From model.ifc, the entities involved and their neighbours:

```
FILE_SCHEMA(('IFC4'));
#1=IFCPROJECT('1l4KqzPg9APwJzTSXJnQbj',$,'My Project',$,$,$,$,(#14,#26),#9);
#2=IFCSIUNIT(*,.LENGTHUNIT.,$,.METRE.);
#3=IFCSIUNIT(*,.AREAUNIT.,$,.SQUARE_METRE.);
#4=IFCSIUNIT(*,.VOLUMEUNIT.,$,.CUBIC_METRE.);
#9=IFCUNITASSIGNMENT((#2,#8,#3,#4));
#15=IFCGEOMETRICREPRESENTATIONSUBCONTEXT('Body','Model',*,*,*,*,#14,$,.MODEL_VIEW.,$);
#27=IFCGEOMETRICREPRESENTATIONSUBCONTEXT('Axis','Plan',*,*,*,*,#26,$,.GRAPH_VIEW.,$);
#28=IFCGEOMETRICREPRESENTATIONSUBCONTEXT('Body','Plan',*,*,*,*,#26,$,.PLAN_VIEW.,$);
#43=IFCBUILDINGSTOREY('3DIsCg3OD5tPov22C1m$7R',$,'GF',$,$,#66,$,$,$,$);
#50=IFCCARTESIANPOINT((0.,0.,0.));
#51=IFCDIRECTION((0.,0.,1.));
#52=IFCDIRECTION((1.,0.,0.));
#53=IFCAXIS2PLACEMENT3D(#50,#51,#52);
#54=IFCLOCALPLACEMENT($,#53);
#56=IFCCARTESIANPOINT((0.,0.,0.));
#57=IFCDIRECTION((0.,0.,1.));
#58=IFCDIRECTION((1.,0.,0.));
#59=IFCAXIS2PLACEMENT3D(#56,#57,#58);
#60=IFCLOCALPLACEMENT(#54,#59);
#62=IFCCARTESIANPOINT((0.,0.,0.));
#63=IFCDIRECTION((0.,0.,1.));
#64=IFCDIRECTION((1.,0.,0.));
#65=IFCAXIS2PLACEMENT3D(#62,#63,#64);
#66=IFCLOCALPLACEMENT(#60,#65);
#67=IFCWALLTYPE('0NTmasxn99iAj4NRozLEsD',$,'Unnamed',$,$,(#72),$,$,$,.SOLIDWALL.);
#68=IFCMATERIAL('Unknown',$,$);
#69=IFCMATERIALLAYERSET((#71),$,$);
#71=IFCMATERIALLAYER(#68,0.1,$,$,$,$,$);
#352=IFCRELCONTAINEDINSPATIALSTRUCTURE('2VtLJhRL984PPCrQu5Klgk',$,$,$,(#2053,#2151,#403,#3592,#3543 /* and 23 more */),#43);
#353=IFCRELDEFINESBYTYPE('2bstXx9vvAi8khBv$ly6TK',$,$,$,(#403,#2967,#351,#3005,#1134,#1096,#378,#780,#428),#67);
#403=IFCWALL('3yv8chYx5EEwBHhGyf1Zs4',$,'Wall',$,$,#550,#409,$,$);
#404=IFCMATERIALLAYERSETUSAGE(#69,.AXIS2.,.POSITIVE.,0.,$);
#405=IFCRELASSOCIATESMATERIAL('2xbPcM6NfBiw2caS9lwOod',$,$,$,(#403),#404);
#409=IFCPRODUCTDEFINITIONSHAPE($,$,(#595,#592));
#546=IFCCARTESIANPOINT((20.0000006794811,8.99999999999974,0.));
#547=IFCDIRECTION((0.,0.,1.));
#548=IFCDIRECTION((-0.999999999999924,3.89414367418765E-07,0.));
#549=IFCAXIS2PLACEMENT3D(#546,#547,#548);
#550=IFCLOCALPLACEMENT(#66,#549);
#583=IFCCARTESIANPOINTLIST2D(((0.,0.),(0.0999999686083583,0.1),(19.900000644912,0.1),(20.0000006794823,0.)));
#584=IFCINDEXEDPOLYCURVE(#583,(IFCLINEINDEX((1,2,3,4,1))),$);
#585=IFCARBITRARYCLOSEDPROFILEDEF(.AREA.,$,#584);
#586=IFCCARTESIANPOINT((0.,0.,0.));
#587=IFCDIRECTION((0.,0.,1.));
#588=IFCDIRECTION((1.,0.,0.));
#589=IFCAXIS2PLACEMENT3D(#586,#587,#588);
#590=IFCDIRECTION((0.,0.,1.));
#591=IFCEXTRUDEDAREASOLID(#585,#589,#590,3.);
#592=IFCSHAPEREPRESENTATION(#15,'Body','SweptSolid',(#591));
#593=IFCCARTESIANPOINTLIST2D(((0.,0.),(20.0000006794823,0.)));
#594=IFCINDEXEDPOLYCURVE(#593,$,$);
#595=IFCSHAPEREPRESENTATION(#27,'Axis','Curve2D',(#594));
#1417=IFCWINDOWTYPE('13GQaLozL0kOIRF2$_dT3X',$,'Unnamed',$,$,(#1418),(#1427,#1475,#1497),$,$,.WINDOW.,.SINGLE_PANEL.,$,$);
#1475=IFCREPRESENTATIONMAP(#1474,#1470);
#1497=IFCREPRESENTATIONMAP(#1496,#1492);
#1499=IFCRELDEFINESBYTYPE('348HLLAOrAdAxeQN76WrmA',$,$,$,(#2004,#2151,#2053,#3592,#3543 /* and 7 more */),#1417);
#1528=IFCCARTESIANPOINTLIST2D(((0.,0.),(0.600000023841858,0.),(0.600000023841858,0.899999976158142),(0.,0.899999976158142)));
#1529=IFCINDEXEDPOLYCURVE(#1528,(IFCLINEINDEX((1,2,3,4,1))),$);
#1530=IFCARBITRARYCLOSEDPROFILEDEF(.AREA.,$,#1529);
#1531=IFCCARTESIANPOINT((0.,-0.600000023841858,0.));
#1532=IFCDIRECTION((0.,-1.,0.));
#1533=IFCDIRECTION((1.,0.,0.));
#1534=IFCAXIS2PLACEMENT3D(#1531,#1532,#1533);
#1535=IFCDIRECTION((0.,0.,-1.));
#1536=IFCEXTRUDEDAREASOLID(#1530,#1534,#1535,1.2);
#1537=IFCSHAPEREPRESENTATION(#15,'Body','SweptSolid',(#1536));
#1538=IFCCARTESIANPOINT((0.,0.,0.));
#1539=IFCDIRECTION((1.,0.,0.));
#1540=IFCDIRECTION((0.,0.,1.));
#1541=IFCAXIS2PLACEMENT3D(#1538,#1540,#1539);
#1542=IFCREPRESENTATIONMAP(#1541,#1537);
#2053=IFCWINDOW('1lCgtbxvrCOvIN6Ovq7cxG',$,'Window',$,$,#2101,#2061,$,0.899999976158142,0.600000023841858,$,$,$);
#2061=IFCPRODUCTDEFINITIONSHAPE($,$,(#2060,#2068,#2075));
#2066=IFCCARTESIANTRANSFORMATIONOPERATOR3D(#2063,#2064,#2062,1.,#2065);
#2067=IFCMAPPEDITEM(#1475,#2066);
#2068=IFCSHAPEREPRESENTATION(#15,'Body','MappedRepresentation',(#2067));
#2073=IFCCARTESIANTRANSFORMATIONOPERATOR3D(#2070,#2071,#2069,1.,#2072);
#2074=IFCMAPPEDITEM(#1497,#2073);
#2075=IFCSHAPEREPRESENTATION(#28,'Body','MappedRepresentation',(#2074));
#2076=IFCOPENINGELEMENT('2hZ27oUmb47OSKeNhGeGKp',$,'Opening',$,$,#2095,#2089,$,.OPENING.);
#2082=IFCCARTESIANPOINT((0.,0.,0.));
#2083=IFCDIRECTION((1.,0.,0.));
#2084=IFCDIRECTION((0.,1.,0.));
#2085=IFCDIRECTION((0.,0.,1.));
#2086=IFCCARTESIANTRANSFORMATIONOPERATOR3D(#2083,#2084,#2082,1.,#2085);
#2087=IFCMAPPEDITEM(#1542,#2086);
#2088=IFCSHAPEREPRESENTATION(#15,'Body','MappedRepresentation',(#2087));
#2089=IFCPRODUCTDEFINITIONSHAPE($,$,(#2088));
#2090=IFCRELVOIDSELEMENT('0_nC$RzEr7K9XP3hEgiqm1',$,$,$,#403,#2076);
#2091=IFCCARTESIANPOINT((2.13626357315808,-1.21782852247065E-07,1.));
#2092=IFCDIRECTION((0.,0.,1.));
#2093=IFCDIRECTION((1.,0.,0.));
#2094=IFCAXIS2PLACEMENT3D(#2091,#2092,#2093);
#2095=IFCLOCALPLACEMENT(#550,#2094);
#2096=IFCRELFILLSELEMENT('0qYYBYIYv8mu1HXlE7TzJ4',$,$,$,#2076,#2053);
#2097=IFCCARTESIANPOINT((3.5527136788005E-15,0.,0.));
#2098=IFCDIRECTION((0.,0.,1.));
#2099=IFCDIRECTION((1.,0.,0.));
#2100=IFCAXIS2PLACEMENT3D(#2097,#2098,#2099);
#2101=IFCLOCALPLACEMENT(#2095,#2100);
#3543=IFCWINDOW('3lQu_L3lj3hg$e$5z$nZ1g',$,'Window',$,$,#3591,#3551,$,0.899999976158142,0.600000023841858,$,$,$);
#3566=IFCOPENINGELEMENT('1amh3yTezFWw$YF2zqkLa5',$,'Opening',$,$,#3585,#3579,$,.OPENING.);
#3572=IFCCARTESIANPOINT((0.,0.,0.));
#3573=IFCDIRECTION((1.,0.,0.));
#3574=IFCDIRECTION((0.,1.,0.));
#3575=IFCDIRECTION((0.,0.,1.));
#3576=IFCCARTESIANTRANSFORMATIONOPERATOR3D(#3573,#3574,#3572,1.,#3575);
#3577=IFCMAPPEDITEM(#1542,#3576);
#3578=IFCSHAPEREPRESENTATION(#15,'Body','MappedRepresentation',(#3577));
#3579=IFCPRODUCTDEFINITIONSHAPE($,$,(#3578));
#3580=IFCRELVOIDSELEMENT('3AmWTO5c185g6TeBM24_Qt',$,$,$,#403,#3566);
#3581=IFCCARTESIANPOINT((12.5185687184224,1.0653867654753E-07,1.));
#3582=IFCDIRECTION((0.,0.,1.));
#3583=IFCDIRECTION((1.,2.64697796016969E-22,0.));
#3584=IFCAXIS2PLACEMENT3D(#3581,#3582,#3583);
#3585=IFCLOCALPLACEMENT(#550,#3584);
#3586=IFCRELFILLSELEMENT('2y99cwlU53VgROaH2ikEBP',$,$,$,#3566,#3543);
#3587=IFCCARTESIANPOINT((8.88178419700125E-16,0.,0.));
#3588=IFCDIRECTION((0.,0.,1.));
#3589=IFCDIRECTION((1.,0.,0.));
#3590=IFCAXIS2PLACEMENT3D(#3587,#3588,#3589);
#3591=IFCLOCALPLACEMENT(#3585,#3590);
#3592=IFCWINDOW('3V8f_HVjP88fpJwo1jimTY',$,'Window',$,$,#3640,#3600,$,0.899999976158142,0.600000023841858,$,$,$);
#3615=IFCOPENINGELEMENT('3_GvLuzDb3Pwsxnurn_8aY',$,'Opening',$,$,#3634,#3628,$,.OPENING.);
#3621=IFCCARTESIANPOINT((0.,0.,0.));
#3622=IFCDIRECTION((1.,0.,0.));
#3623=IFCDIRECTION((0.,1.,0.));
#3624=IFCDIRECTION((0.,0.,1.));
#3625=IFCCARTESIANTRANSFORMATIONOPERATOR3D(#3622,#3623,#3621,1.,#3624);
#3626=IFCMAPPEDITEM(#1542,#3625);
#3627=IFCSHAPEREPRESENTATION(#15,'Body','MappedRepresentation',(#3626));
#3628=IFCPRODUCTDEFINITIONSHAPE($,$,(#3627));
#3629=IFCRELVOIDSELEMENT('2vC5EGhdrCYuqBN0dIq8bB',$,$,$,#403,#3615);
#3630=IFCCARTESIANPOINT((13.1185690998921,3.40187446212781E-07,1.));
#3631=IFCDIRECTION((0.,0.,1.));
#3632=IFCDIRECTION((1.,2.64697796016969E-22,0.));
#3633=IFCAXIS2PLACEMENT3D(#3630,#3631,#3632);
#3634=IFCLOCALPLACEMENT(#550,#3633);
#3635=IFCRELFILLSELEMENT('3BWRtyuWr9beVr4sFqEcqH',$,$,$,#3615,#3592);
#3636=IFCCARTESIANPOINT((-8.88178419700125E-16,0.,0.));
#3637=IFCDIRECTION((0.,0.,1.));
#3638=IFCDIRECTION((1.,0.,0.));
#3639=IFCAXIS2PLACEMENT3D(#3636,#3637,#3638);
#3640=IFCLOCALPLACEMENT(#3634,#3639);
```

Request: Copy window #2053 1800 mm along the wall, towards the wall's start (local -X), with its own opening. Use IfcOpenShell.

```python
import ifcopenshell
import ifcopenshell.api.feature
import ifcopenshell.api.geometry
import ifcopenshell.api.root
import ifcopenshell.geom
import ifcopenshell.util.element
import ifcopenshell.util.placement
import ifcopenshell.util.shape

model = ifcopenshell.open("model.ifc")
settings = ifcopenshell.geom.settings()


def volume(element):
    """Net volume in cubic metres, openings subtracted."""
    shape = ifcopenshell.geom.create_shape(settings, element)
    return ifcopenshell.util.shape.get_volume(shape.geometry)


window = model.by_guid("1lCgtbxvrCOvIN6Ovq7cxG")
opening = window.FillsVoids[0].RelatingOpeningElement
wall = opening.VoidsElements[0].RelatingBuildingElement
before = volume(wall)
shift = ifcopenshell.util.placement.get_local_placement(wall.ObjectPlacement)[:3, 0] * -1.8

# copy_class copies the void relationship, type, container and properties, but no geometry.
new_opening = ifcopenshell.api.root.copy_class(model, product=opening)
new_opening.Representation = ifcopenshell.util.element.copy_deep(
    model, opening.Representation, exclude=["IfcGeometricRepresentationContext", "IfcRepresentationMap"]
)
new_window = ifcopenshell.api.root.copy_class(model, product=window)
new_window.Representation = ifcopenshell.util.element.copy_deep(
    model, window.Representation, exclude=["IfcGeometricRepresentationContext", "IfcRepresentationMap"]
)
ifcopenshell.api.feature.add_filling(model, opening=new_opening, element=new_window)

for old, new in ((opening, new_opening), (window, new_window)):
    matrix = ifcopenshell.util.placement.get_local_placement(old.ObjectPlacement)
    matrix[:3, 3] += shift
    ifcopenshell.api.geometry.edit_object_placement(model, product=new, matrix=matrix, is_si=False)

after = volume(wall)

print(f"wall volume {before:.3f} -> {after:.3f} m3")

model.write("model_edited.ifc")
```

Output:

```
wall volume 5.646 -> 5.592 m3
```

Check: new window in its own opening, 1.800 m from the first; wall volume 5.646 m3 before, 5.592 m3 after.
